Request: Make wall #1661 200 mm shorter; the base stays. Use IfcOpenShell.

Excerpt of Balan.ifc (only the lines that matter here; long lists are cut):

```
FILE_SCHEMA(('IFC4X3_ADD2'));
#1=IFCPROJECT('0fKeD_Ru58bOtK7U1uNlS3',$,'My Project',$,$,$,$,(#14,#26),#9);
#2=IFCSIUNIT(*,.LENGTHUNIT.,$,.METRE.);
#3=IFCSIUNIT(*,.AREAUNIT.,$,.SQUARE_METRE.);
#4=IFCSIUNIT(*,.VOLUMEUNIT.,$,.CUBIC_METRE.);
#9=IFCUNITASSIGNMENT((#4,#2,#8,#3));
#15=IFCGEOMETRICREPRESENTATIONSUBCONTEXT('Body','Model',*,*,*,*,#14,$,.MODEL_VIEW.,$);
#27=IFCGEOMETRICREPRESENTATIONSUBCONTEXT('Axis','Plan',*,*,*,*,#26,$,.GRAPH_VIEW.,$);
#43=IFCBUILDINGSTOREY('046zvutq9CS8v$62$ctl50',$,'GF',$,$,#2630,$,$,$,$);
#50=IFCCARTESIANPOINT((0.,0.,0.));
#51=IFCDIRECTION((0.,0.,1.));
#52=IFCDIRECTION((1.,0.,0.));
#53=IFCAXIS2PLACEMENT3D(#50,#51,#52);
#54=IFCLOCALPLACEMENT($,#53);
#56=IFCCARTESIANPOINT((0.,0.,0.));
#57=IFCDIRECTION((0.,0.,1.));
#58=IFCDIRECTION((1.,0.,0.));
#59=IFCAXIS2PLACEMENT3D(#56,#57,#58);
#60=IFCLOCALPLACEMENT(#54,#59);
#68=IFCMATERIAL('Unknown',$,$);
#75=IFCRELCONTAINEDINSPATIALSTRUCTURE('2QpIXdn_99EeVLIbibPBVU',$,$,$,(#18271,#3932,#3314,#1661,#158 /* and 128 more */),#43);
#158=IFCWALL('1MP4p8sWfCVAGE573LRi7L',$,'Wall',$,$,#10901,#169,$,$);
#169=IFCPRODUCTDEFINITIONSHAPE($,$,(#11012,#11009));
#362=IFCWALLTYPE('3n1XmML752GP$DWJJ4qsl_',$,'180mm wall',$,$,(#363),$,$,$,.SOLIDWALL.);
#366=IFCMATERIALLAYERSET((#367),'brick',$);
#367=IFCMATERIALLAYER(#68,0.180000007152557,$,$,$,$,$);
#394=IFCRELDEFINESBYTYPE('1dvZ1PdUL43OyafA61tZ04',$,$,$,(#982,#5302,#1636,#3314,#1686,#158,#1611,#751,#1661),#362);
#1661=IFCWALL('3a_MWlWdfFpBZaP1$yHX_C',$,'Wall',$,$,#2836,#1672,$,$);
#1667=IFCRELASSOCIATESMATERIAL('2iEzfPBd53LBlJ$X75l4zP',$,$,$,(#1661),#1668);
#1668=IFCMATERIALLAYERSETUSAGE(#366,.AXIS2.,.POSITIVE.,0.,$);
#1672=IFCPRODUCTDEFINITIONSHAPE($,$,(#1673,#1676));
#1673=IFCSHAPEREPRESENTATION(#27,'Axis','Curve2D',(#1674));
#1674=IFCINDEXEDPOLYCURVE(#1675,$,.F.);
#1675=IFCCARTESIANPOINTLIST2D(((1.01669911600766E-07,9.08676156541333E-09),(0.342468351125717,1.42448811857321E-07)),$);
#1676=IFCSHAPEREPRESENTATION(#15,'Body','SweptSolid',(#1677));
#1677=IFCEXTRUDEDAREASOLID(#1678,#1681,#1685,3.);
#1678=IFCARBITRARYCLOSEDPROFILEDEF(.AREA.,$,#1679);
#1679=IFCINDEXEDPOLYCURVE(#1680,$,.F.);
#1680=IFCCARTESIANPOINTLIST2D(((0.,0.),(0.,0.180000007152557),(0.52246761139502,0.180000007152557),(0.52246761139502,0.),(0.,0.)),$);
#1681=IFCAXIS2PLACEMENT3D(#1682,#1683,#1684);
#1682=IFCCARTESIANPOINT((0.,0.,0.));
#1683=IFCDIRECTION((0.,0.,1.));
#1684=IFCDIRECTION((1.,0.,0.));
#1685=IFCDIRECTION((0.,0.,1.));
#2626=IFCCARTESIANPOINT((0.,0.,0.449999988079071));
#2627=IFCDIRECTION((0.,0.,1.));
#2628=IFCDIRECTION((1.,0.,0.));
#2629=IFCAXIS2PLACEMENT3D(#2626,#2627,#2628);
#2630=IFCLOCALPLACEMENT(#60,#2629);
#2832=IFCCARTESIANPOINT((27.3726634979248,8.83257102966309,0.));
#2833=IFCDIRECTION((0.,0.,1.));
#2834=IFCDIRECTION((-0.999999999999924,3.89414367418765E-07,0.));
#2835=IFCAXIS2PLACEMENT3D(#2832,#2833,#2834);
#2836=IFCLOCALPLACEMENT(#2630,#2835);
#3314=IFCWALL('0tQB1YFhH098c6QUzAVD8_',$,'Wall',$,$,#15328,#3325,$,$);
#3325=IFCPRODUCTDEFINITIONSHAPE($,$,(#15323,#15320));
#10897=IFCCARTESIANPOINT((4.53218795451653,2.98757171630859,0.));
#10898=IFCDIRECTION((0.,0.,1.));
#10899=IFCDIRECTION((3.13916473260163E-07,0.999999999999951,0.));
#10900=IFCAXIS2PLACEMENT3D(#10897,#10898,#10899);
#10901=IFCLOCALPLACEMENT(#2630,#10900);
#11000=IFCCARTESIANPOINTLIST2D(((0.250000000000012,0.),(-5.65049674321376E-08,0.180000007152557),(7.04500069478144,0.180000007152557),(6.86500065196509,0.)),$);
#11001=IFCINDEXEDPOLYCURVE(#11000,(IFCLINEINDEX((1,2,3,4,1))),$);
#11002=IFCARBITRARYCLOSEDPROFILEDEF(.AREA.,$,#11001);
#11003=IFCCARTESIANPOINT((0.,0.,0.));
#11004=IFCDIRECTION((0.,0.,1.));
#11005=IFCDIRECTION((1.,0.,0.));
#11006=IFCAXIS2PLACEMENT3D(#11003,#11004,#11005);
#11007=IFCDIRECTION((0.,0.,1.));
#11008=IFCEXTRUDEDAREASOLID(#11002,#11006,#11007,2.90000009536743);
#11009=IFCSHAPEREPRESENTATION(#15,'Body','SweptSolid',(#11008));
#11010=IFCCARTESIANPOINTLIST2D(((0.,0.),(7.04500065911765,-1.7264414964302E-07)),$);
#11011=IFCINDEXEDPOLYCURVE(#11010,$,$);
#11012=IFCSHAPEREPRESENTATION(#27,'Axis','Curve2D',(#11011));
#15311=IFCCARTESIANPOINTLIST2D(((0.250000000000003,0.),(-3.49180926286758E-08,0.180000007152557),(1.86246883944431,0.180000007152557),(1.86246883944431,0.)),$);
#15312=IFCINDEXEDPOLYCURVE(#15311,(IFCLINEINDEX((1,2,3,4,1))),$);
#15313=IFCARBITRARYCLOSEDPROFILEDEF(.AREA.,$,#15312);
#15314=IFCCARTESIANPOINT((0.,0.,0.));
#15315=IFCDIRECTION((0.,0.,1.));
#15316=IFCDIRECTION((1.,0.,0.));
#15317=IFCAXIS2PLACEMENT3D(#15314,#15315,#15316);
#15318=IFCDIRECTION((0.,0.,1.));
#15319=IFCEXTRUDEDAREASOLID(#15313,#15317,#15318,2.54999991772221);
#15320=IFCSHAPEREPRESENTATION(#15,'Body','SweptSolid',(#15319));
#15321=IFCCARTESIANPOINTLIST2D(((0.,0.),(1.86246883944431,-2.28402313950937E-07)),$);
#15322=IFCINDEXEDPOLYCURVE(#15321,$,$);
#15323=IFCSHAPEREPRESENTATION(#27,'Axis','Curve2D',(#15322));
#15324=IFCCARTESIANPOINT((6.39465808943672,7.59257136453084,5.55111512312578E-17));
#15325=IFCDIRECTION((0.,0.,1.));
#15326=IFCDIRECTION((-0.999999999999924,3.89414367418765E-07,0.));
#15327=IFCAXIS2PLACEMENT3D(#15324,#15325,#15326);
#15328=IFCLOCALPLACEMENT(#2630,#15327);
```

```python
import ifcopenshell
import ifcopenshell.geom
import ifcopenshell.util.representation
import ifcopenshell.util.shape

model = ifcopenshell.open("Balan.ifc")
settings = ifcopenshell.geom.settings()


def volume(element):
    """Net volume in cubic metres, openings subtracted."""
    shape = ifcopenshell.geom.create_shape(settings, element)
    return ifcopenshell.util.shape.get_volume(shape.geometry)


wall = model.by_guid("3a_MWlWdfFpBZaP1$yHX_C")
before = volume(wall)

body = ifcopenshell.util.representation.get_representation(wall, "Model", "Body")
solid = body.Items[0]
old_height = solid.Depth
solid.Depth -= 0.2
after = volume(wall)

print(f"height {old_height:g} -> {solid.Depth:g}, volume {before:.3f} -> {after:.3f} m3")

model.write("Balan_v2.ifc")
```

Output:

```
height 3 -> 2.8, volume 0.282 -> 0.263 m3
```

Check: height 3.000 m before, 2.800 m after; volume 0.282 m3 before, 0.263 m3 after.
